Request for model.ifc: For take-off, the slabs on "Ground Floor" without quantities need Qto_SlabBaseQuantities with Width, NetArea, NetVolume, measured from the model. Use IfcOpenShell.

First a look at what the model holds.

```python
import ifcopenshell
import ifcopenshell.util.element
import ifcopenshell.util.unit

model = ifcopenshell.open("model.ifc")
print(model.schema)
for unit_type in ("LENGTHUNIT", "AREAUNIT", "VOLUMEUNIT"):
    print(unit_type, ifcopenshell.util.unit.calculate_unit_scale(model, unit_type))
storey = next(s for s in model.by_type("IfcBuildingStorey") if s.Name == "Ground Floor")
slabs = [e for e in ifcopenshell.util.element.get_decomposition(storey) if e.is_a("IfcSlab")]
for e in sorted(slabs, key=lambda e: e.id()):
    print(e.id(), e.is_a(), e.Name, list(ifcopenshell.util.element.get_psets(e, qtos_only=True)), sep=" | ")
```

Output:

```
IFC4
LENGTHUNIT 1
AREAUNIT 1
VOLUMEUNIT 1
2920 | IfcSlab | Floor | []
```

```python
import ifcopenshell
import ifcopenshell.api.pset
import ifcopenshell.geom
import ifcopenshell.util.element
import ifcopenshell.util.shape
import ifcopenshell.util.unit

model = ifcopenshell.open("model.ifc")
unit_scale = ifcopenshell.util.unit.calculate_unit_scale(model)
area_scale = ifcopenshell.util.unit.calculate_unit_scale(model, "AREAUNIT")
volume_scale = ifcopenshell.util.unit.calculate_unit_scale(model, "VOLUMEUNIT")
settings = ifcopenshell.geom.settings()

storey = next(s for s in model.by_type("IfcBuildingStorey") if s.Name == "Ground Floor")
slabs = [e for e in ifcopenshell.util.element.get_decomposition(storey) if e.is_a("IfcSlab")]

for e in sorted(slabs, key=lambda e: e.id()):
    if ifcopenshell.util.element.get_psets(e, qtos_only=True, should_inherit=False):
        continue
    # Geometry comes back in metres, in the element's own axes.
    shape = ifcopenshell.geom.create_shape(settings, e)
    values = {
        "Width": ifcopenshell.util.shape.get_z(shape.geometry) / unit_scale,
        "NetArea": ifcopenshell.util.shape.get_footprint_area(shape.geometry) / area_scale,
        "NetVolume": ifcopenshell.util.shape.get_volume(shape.geometry) / volume_scale,
    }
    qto = ifcopenshell.api.pset.add_qto(model, product=e, name="Qto_SlabBaseQuantities")
    ifcopenshell.api.pset.edit_qto(model, qto=qto, properties=values)
    print(e.id(), {k: round(v, 3) for k, v in values.items()})

model.write("model-out.ifc")
```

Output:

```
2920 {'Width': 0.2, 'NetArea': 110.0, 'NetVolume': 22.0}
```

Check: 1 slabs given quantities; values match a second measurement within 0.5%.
